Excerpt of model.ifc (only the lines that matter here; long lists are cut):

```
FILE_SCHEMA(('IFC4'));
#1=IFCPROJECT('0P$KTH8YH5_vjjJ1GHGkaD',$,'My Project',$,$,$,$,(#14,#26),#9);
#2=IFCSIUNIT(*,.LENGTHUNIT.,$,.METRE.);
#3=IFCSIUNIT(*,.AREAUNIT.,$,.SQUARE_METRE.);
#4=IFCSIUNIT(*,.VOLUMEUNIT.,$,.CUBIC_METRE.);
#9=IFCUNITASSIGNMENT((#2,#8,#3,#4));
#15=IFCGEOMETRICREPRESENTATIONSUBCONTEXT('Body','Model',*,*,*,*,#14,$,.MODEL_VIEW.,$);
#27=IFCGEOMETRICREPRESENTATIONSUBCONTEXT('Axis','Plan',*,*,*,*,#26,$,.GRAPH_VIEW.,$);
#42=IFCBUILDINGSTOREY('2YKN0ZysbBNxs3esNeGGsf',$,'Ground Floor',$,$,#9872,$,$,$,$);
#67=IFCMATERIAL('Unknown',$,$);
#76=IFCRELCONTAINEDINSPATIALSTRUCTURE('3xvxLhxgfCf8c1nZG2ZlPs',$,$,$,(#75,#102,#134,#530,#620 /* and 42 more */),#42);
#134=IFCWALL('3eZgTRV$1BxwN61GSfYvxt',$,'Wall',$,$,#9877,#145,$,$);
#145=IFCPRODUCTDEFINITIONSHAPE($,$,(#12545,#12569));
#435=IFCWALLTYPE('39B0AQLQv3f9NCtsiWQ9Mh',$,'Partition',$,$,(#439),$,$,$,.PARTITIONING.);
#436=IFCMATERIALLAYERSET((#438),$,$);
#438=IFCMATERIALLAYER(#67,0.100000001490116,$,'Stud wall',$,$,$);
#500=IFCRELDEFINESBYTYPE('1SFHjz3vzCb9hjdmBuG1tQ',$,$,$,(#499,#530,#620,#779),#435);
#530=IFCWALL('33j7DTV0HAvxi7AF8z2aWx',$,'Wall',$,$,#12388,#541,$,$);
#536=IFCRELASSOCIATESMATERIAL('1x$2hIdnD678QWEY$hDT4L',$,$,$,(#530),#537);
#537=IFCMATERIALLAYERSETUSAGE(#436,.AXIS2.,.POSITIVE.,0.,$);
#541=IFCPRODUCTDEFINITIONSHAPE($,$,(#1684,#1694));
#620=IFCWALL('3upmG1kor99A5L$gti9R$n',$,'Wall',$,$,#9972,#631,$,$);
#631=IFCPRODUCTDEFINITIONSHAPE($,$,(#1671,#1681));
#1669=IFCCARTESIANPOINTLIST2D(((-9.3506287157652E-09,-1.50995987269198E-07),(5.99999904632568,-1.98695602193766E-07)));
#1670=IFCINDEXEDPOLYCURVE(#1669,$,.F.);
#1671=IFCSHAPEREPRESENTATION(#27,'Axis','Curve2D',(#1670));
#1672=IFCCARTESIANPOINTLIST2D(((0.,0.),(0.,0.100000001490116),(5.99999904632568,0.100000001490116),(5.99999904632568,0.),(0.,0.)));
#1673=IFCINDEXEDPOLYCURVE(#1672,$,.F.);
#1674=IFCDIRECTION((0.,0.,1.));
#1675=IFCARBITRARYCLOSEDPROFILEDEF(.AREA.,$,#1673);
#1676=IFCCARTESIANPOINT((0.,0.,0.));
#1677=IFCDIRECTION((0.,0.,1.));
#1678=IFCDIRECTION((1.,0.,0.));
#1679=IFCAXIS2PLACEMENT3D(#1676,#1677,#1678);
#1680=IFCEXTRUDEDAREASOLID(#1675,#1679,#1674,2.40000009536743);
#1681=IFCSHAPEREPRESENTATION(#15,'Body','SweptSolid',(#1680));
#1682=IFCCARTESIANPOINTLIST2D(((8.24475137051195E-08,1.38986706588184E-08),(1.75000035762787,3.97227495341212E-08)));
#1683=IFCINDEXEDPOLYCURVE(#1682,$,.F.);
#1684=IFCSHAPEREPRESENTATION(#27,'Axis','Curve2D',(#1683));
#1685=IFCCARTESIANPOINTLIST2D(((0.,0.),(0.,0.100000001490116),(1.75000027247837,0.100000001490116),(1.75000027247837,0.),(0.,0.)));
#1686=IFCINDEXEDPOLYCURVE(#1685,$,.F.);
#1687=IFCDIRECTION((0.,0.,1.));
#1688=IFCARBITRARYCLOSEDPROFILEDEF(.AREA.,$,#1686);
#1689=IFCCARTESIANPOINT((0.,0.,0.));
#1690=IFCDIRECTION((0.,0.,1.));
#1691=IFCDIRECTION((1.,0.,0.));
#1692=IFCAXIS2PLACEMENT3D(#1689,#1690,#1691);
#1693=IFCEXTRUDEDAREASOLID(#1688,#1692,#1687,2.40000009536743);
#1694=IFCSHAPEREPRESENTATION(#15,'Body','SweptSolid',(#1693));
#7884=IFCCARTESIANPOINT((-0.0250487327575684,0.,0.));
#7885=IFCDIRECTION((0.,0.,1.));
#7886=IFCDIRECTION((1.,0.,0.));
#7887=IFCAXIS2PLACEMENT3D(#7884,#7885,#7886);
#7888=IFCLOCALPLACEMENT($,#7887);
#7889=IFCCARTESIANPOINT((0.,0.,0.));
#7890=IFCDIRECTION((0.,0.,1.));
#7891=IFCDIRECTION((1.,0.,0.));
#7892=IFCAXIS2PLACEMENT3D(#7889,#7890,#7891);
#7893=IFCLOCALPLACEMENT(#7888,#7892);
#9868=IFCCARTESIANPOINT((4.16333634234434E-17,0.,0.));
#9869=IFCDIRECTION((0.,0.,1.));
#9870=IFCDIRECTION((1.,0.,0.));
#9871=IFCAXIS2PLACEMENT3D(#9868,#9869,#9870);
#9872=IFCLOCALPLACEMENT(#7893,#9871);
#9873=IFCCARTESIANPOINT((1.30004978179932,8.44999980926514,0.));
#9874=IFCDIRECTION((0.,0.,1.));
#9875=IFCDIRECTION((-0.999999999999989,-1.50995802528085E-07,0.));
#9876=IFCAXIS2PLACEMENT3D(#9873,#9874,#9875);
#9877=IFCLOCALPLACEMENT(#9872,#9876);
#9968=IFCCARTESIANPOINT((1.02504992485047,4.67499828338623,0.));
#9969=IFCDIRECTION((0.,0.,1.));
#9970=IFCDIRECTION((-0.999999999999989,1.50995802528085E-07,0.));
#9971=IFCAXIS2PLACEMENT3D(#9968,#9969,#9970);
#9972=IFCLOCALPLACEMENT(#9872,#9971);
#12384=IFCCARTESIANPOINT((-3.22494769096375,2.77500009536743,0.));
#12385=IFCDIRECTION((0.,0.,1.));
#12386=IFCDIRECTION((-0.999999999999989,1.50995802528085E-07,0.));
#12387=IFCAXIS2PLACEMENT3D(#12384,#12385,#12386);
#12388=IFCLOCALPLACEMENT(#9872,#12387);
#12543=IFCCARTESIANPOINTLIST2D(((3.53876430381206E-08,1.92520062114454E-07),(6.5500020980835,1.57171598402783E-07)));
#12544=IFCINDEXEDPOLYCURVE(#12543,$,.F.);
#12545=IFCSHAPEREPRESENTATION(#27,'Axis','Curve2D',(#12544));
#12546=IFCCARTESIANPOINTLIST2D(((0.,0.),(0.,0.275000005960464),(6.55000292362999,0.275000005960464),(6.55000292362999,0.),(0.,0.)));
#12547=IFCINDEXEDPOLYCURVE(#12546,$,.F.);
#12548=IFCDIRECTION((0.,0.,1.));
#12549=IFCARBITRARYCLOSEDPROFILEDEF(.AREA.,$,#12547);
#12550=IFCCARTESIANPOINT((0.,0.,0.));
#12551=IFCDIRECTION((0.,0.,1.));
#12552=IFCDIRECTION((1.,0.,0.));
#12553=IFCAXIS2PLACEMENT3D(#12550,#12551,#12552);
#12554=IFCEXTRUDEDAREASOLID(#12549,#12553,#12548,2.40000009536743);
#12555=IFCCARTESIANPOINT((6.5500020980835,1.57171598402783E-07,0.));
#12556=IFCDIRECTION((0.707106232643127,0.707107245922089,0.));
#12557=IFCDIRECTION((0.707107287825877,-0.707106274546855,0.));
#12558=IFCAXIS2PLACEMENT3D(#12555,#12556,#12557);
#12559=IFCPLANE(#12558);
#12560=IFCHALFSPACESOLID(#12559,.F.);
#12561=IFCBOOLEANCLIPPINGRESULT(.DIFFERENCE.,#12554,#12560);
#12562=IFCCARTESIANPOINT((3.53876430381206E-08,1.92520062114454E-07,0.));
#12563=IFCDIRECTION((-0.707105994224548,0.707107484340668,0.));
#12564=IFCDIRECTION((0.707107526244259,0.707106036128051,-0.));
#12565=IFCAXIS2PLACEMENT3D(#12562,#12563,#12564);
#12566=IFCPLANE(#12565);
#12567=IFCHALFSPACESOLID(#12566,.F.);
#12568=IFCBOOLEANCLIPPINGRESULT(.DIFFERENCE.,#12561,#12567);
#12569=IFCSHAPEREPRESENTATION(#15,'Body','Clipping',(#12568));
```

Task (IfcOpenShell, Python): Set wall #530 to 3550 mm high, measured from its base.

```python
import ifcopenshell
import ifcopenshell.geom
import ifcopenshell.util.representation
import ifcopenshell.util.shape
import ifcopenshell.util.unit

model = ifcopenshell.open("model.ifc")
unit_scale = ifcopenshell.util.unit.calculate_unit_scale(model)
settings = ifcopenshell.geom.settings()


def volume(element):
    """Net volume in cubic metres, openings subtracted."""
    shape = ifcopenshell.geom.create_shape(settings, element)
    return ifcopenshell.util.shape.get_volume(shape.geometry)


wall = model.by_guid("33j7DTV0HAvxi7AF8z2aWx")
before = volume(wall)

body = ifcopenshell.util.representation.get_representation(wall, "Model", "Body")
solid = body.Items[0]
old_height = solid.Depth
solid.Depth = 3.55 / unit_scale
after = volume(wall)

print(f"height {old_height:g} -> {solid.Depth:g}, volume {before:.3f} -> {after:.3f} m3")

model.write("model_rev.ifc")
```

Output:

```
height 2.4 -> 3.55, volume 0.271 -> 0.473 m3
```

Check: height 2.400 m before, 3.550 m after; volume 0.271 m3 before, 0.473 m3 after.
